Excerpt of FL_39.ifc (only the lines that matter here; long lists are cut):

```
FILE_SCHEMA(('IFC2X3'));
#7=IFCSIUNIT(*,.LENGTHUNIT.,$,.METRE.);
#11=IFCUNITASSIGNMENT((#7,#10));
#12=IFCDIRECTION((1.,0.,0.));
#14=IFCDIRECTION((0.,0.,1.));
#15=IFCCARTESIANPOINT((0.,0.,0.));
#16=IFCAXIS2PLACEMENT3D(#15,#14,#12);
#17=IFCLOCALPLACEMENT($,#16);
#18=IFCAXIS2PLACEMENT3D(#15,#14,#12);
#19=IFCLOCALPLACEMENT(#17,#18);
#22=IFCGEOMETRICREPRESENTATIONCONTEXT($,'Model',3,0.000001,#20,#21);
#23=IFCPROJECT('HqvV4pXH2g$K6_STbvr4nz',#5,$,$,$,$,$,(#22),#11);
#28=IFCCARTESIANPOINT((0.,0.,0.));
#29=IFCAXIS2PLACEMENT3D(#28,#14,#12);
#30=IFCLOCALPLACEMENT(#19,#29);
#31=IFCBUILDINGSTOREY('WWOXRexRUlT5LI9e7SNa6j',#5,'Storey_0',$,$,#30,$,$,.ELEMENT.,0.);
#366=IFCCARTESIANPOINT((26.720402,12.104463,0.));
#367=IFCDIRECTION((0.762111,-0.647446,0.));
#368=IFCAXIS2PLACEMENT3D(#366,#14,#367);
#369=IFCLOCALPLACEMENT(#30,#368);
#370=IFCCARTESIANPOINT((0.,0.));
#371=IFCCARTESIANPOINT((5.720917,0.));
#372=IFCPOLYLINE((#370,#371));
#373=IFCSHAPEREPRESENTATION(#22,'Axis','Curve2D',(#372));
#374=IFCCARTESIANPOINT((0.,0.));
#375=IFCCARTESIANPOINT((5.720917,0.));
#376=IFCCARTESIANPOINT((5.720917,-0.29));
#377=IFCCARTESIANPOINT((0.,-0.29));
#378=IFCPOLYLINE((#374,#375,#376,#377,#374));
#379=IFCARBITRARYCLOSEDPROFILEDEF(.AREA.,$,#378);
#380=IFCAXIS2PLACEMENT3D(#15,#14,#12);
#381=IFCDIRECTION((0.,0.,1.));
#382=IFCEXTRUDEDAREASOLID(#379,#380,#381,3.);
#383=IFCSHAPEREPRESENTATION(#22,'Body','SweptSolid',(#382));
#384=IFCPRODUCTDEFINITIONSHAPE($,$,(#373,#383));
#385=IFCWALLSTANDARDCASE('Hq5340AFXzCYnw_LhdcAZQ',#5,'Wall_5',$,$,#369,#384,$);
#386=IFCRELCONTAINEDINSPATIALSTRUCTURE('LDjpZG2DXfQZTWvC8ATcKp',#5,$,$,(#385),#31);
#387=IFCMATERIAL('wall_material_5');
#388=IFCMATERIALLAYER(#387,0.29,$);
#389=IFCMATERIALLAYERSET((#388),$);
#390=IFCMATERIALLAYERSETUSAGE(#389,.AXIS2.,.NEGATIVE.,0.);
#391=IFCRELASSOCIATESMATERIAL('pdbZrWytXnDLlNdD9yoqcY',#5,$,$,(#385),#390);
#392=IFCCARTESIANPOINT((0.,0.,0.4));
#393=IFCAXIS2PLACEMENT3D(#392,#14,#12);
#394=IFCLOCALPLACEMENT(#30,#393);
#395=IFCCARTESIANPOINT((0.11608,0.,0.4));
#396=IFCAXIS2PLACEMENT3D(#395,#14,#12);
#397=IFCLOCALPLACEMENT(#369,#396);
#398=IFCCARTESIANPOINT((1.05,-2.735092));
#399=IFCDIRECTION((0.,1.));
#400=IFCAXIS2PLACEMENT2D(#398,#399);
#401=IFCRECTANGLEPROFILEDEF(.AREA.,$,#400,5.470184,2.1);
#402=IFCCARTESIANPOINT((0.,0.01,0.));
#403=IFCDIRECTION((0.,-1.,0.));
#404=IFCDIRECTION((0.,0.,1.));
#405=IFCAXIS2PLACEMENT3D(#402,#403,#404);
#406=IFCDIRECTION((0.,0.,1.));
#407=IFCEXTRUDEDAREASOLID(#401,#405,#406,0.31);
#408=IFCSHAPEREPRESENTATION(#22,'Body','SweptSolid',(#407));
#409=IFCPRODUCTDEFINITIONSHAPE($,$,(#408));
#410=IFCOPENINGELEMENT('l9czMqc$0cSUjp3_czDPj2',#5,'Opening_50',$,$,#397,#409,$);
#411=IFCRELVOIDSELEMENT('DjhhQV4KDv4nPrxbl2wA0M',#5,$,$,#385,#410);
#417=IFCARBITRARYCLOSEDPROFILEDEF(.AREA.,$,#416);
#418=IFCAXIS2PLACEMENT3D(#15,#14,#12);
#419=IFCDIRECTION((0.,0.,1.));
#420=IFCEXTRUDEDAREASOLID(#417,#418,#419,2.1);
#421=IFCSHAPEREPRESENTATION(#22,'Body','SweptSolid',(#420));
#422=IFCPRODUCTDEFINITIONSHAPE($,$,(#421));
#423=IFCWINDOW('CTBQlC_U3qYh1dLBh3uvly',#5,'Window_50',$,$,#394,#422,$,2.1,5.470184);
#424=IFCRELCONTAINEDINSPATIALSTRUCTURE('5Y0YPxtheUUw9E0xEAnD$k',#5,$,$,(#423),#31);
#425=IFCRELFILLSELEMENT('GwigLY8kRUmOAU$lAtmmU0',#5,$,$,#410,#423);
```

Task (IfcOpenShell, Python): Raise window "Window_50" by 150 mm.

```python
import numpy as np
import ifcopenshell
import ifcopenshell.api.geometry
import ifcopenshell.util.placement
import ifcopenshell.util.unit

model = ifcopenshell.open("FL_39.ifc")
unit_scale = ifcopenshell.util.unit.calculate_unit_scale(model)

window = model.by_guid("CTBQlC_U3qYh1dLBh3uvly")
opening = window.FillsVoids[0].RelatingOpeningElement
dz = 0.15 / unit_scale

shift = np.array([0.0, 0.0, dz])
# The window is not placed relative to its opening, so move both.
for product in (opening, window):
    matrix = ifcopenshell.util.placement.get_local_placement(product.ObjectPlacement)
    matrix[:3, 3] += shift
    ifcopenshell.api.geometry.edit_object_placement(model, product=product, matrix=matrix, is_si=False)

print(f"moved by {dz * unit_scale:+.3f} m")

model.write("FL_39_updated.ifc")
```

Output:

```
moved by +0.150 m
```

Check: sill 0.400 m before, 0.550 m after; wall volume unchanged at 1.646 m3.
